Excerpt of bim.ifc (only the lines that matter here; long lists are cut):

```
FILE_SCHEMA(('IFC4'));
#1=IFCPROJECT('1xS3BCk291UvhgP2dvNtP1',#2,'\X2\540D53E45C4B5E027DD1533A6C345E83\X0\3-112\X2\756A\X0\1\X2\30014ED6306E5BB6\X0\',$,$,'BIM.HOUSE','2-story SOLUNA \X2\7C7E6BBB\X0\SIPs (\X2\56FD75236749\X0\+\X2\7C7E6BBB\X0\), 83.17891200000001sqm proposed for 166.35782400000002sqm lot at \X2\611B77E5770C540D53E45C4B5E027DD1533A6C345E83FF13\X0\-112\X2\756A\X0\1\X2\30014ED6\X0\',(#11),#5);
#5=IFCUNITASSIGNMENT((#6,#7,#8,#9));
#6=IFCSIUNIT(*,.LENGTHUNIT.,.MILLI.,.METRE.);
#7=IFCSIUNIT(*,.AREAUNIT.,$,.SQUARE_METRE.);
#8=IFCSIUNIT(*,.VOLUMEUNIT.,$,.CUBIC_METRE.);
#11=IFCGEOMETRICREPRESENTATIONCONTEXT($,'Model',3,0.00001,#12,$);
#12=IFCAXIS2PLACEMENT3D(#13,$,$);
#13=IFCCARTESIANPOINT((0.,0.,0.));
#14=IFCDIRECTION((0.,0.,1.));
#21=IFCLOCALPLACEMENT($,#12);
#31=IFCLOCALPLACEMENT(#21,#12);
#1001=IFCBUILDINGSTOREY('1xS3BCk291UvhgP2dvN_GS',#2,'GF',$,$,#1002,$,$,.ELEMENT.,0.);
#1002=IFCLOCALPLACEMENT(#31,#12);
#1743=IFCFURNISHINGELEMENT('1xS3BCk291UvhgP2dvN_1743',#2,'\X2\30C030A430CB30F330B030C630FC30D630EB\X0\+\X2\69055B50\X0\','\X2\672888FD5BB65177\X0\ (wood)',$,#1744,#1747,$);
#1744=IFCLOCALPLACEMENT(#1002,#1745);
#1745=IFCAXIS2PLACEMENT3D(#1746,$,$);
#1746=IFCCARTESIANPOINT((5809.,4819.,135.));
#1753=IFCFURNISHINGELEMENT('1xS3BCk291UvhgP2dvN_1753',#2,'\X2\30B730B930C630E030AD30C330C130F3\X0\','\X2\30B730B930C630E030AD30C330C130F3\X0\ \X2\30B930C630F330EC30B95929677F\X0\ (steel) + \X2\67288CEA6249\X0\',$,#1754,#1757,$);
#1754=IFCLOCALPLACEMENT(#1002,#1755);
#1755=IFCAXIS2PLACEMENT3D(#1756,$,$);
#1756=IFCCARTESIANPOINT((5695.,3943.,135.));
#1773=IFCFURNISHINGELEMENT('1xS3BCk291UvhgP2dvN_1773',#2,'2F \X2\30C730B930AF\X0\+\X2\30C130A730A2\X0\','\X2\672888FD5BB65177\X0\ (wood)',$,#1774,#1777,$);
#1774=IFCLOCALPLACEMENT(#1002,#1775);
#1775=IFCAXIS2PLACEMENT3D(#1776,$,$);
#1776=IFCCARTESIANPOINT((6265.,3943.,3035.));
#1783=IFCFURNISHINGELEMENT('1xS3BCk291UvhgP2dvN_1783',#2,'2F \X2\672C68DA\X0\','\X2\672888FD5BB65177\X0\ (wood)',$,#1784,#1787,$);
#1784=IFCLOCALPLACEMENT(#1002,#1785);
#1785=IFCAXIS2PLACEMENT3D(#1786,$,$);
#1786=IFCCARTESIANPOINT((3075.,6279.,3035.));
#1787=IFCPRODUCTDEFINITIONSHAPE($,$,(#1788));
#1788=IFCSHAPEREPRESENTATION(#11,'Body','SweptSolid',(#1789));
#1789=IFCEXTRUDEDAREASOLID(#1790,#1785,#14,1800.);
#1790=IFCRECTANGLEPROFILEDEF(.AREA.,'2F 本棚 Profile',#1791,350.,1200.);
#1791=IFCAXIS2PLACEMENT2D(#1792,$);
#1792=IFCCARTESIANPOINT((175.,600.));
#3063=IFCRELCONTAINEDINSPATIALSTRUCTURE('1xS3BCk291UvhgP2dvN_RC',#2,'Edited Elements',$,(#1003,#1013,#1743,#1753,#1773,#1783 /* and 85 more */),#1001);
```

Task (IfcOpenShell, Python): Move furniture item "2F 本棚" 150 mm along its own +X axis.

```python
import ifcopenshell
import ifcopenshell.api.geometry
import ifcopenshell.util.placement
import ifcopenshell.util.unit

model = ifcopenshell.open("bim.ifc")
unit_scale = ifcopenshell.util.unit.calculate_unit_scale(model)

item = model.by_id(1783)
matrix = ifcopenshell.util.placement.get_local_placement(item.ObjectPlacement)
matrix[:3, 3] += matrix[:3, 0] * 0.15 / unit_scale
ifcopenshell.api.geometry.edit_object_placement(model, product=item, matrix=matrix, is_si=False)

print(ifcopenshell.util.placement.get_local_placement(item.ObjectPlacement).round(3) + 0.0)

model.write("bim_rev.ifc")
```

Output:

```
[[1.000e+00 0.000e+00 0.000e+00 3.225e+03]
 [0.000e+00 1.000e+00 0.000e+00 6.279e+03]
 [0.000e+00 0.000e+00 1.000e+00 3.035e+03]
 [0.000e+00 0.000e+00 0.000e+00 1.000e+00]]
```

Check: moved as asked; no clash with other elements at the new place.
